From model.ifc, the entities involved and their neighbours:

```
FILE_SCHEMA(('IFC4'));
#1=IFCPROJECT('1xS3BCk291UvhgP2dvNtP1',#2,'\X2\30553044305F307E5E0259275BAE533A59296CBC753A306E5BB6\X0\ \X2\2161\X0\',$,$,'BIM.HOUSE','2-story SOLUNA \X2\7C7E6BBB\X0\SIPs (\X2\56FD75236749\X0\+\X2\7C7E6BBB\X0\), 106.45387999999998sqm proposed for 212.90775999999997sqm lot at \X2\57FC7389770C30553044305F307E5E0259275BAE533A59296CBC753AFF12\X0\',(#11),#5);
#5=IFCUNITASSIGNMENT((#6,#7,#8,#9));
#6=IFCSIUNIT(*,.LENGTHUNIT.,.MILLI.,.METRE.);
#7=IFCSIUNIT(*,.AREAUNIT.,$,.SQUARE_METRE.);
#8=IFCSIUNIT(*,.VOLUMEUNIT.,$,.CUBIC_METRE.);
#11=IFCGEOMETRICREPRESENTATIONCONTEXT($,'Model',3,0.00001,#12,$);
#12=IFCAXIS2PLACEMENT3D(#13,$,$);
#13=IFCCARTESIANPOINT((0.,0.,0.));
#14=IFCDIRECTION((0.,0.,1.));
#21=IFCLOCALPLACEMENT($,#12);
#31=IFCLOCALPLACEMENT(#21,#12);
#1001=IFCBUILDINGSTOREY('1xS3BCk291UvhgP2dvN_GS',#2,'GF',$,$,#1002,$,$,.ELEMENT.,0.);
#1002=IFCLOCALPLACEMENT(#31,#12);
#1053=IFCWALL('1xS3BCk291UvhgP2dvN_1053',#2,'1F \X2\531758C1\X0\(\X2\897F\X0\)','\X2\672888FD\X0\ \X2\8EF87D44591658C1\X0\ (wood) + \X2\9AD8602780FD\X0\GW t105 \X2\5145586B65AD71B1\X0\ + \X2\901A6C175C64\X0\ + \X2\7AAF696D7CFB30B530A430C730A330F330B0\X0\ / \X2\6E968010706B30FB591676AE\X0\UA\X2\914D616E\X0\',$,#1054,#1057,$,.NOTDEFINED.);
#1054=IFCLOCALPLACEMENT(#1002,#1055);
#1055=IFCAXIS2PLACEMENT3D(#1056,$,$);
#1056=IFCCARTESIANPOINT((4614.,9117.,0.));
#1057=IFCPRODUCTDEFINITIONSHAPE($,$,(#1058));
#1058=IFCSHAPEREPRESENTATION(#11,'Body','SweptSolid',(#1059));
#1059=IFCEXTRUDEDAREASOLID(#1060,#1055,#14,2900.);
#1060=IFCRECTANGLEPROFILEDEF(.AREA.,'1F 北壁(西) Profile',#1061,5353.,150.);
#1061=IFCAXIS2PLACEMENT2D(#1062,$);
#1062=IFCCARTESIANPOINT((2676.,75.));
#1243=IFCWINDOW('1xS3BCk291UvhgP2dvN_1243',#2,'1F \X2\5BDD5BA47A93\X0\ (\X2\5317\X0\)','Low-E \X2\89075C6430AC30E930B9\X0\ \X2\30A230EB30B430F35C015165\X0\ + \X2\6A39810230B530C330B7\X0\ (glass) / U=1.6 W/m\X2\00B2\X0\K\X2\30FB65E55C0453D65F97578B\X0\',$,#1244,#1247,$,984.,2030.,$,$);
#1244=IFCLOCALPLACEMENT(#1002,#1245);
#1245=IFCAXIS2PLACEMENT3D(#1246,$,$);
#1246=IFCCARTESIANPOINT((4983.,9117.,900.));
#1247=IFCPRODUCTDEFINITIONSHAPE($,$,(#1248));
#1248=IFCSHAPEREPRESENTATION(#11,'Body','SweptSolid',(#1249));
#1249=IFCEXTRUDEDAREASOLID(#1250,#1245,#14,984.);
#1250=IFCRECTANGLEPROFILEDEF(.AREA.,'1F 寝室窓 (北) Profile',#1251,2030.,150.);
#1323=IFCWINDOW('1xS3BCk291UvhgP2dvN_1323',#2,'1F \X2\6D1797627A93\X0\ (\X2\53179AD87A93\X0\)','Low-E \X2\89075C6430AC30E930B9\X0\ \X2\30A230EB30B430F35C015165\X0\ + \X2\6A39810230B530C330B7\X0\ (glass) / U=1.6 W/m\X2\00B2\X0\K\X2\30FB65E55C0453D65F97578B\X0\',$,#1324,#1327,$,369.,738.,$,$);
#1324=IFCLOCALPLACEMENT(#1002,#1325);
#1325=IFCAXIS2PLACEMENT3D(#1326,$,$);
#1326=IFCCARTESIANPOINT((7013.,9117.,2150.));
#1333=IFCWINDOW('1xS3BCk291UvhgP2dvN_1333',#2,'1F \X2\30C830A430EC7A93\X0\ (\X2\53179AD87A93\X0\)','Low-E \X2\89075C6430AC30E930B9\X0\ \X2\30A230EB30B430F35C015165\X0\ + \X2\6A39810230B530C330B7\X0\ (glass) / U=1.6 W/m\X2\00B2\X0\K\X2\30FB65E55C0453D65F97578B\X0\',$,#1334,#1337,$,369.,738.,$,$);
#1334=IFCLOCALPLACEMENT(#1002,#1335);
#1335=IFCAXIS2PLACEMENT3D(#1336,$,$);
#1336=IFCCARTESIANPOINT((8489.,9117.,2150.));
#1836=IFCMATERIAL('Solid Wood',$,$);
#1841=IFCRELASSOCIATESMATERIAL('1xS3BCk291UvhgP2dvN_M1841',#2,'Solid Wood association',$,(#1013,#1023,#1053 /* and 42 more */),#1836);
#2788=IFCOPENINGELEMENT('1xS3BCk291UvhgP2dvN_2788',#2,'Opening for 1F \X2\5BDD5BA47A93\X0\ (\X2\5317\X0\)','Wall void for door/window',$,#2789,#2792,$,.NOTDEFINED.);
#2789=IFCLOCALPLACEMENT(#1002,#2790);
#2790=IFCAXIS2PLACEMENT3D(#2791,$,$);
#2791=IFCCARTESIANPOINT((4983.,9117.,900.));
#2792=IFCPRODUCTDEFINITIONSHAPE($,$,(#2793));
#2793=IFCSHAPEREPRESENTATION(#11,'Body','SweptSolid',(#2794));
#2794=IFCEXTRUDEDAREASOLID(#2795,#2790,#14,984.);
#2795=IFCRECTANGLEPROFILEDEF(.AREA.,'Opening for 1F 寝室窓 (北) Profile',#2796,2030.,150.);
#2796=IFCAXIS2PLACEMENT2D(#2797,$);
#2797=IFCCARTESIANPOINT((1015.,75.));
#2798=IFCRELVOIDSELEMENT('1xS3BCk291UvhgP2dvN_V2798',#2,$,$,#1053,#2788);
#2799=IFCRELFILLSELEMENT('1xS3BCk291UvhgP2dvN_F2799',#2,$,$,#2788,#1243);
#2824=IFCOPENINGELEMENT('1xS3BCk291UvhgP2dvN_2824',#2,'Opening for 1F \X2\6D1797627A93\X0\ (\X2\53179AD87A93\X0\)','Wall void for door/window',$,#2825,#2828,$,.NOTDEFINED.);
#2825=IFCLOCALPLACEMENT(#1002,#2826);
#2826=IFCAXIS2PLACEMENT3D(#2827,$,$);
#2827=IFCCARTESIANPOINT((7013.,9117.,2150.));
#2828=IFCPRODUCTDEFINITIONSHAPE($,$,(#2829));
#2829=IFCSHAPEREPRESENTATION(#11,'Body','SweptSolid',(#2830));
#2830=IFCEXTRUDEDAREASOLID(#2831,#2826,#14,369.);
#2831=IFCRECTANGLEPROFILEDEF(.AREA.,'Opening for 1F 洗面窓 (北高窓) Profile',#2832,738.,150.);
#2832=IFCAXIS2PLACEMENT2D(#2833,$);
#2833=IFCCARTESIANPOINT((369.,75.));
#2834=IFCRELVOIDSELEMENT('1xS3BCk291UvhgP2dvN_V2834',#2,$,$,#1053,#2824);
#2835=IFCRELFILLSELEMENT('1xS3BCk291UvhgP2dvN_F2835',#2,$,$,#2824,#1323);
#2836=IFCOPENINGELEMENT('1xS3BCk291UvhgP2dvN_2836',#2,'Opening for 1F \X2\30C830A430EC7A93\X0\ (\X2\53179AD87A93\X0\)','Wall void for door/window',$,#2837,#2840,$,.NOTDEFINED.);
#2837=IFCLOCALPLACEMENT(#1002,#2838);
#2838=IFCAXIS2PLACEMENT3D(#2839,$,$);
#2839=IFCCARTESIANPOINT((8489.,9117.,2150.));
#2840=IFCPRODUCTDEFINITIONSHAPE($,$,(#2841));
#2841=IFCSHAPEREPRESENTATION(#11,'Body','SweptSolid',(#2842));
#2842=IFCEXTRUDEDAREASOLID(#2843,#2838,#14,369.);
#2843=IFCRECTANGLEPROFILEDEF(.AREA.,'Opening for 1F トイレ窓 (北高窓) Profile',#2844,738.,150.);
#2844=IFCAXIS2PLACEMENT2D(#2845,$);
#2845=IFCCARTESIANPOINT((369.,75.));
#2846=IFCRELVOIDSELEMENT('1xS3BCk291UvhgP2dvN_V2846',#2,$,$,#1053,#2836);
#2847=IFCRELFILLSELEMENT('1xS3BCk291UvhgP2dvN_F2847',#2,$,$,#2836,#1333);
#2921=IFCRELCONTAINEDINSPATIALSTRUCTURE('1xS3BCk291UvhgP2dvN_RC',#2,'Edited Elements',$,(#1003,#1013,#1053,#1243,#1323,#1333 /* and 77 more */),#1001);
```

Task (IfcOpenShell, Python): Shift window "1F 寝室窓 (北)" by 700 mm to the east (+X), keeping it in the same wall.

```python
import ifcopenshell
import ifcopenshell.api.geometry
import ifcopenshell.util.placement

model = ifcopenshell.open("model.ifc")

window = model.by_guid("1xS3BCk291UvhgP2dvN_1243")
opening = window.FillsVoids[0].RelatingOpeningElement
wall = opening.VoidsElements[0].RelatingBuildingElement

wall_matrix = ifcopenshell.util.placement.get_local_placement(wall.ObjectPlacement)
shift = wall_matrix[:3, 0] * 700.0
before = ifcopenshell.util.placement.get_local_placement(window.ObjectPlacement)[:3, 3].copy()

# The window is not placed relative to its opening, so move both.
for product in (opening, window):
    matrix = ifcopenshell.util.placement.get_local_placement(product.ObjectPlacement)
    matrix[:3, 3] += shift
    ifcopenshell.api.geometry.edit_object_placement(model, product=product, matrix=matrix, is_si=False)

after = ifcopenshell.util.placement.get_local_placement(window.ObjectPlacement)[:3, 3]
print("window moved by", (after - before).round(3) + 0.0)

model.write("model_updated.ifc")
```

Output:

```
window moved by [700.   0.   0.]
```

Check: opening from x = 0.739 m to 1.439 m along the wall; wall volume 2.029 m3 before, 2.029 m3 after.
